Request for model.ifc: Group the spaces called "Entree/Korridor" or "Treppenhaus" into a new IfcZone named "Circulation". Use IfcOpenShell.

First a look at what the model holds.

```python
import ifcopenshell

model = ifcopenshell.open("model.ifc")
print(model.schema)
seen = {}
for space in model.by_type("IfcSpace"):
    seen[space.LongName] = seen.get(space.LongName, 0) + 1
for name, count in sorted(seen.items(), key=str):
    print(count, "x", name)
print("zones:", [z.Name for z in model.by_type("IfcZone")][:20])
```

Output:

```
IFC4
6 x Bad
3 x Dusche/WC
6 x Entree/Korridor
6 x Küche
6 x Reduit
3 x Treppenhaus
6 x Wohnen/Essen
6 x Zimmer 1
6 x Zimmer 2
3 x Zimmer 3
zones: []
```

```python
import ifcopenshell
import ifcopenshell.api.group
import ifcopenshell.api.root

model = ifcopenshell.open("model.ifc")

names = {"Entree/Korridor", "Treppenhaus"}
spaces = [s for s in model.by_type("IfcSpace") if s.LongName in names]

zone = ifcopenshell.api.root.create_entity(model, ifc_class="IfcZone", name="Circulation")
ifcopenshell.api.group.assign_group(model, products=spaces, group=zone)
print(len(spaces), "spaces in", zone.Name)

model.write("model_rev.ifc")
```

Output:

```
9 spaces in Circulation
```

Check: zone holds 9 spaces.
